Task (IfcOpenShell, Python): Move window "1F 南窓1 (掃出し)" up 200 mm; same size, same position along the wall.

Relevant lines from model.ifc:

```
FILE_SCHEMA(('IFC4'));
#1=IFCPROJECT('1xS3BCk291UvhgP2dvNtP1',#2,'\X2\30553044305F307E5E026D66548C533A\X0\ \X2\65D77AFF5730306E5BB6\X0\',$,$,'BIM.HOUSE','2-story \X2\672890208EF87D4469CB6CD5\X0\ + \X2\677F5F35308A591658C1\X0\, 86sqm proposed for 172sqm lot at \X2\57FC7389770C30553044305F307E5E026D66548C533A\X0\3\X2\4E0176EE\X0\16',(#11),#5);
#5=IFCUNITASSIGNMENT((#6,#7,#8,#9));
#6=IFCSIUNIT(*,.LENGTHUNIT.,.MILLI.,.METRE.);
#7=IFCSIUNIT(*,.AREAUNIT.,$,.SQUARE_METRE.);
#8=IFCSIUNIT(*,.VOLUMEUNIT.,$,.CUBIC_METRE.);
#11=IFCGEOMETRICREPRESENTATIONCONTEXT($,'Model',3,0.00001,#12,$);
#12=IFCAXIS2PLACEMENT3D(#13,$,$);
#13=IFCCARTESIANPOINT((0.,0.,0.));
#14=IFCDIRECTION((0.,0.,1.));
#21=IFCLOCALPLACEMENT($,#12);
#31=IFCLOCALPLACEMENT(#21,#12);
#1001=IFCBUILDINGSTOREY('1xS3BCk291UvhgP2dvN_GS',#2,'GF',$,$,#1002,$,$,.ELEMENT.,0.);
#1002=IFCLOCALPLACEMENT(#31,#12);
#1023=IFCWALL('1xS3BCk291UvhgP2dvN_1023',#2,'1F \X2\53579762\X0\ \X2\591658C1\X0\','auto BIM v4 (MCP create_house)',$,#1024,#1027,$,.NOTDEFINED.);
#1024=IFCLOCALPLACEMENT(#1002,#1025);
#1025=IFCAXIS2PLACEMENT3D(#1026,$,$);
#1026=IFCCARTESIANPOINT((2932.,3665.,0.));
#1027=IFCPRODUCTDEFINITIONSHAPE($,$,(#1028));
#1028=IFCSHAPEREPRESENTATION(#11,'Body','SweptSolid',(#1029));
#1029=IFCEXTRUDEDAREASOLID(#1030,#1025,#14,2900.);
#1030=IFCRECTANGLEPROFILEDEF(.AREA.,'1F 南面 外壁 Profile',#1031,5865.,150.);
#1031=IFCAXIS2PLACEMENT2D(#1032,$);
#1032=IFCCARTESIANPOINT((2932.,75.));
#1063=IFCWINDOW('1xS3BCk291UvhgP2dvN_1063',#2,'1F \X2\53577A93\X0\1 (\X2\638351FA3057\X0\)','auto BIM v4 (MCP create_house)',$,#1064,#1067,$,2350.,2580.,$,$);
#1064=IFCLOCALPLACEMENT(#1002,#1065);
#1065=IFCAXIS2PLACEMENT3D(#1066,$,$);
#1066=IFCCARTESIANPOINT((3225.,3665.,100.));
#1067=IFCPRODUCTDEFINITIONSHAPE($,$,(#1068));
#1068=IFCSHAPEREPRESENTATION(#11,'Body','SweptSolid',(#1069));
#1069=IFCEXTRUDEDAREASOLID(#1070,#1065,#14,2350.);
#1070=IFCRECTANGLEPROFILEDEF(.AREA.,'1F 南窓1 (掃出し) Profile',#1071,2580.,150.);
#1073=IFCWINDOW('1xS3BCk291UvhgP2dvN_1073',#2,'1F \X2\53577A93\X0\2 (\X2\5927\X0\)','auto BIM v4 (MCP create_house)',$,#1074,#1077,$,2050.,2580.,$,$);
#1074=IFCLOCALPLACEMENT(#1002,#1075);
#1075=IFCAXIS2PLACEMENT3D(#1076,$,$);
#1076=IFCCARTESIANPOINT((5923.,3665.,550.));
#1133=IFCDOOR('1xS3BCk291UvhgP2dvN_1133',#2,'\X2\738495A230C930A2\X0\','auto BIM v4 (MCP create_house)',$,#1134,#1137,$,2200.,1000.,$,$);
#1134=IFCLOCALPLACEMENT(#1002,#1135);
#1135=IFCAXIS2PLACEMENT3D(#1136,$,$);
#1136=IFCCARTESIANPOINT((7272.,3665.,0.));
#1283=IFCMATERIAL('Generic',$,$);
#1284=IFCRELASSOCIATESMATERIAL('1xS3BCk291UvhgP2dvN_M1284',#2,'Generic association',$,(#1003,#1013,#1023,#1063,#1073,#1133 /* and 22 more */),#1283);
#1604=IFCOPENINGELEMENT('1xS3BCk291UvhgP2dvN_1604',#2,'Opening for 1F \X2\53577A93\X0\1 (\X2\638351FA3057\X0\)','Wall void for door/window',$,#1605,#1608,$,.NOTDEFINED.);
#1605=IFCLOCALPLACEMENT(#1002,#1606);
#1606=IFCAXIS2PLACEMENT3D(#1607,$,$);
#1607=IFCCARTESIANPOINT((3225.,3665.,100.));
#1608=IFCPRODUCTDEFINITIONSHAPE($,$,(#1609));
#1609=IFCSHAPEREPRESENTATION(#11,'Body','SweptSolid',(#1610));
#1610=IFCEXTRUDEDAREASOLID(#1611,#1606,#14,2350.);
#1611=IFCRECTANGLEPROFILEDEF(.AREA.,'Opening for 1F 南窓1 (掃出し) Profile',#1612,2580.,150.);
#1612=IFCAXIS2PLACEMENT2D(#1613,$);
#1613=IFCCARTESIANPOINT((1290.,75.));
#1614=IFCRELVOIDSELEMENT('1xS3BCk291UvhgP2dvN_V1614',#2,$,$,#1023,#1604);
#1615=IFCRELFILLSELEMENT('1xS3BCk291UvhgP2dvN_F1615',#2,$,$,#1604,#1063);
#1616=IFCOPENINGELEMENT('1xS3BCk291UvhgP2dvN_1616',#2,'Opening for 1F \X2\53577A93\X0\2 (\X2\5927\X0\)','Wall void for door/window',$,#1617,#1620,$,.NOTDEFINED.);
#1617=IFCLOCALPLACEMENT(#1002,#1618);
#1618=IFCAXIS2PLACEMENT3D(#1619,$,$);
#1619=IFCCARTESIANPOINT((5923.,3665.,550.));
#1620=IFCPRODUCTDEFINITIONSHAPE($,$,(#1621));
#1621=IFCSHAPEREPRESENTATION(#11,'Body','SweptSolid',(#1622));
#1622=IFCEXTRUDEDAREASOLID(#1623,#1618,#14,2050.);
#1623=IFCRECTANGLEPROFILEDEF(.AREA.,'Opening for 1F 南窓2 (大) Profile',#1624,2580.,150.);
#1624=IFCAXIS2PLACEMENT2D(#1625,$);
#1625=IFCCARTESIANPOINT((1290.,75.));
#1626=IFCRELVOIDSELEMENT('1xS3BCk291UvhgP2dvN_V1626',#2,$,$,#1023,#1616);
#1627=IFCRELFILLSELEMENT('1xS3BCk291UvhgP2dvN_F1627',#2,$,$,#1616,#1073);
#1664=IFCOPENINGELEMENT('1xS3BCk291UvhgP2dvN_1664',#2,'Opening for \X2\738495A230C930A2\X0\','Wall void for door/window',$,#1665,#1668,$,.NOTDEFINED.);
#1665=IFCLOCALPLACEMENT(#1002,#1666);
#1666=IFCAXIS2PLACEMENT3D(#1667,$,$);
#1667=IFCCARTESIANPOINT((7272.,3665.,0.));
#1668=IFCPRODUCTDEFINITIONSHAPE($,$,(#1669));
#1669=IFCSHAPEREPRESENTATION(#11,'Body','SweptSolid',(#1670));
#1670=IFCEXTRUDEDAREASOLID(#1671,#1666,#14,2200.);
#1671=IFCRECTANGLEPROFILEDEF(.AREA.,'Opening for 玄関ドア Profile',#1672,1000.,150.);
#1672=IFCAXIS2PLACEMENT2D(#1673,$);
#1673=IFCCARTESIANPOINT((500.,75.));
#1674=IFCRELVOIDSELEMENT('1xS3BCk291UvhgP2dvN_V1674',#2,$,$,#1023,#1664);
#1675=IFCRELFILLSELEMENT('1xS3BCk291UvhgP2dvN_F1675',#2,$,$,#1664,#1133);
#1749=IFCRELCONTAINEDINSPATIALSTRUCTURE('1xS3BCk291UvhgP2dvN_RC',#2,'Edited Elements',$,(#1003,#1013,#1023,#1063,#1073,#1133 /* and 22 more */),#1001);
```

```python
import numpy as np
import ifcopenshell
import ifcopenshell.api.geometry
import ifcopenshell.util.placement
import ifcopenshell.util.unit

model = ifcopenshell.open("model.ifc")
unit_scale = ifcopenshell.util.unit.calculate_unit_scale(model)

window = model.by_id(1063)
opening = window.FillsVoids[0].RelatingOpeningElement
dz = 0.2 / unit_scale

shift = np.array([0.0, 0.0, dz])
# The window is not placed relative to its opening, so move both.
for product in (opening, window):
    matrix = ifcopenshell.util.placement.get_local_placement(product.ObjectPlacement)
    matrix[:3, 3] += shift
    ifcopenshell.api.geometry.edit_object_placement(model, product=product, matrix=matrix, is_si=False)

print(f"moved by {dz * unit_scale:+.3f} m")

model.write("model_edited.ifc")
```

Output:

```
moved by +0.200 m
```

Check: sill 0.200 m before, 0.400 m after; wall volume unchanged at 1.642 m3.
